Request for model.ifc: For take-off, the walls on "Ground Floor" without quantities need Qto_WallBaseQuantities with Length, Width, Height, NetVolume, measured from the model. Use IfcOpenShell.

First a look at what the model holds.

```python
import ifcopenshell
import ifcopenshell.util.element
import ifcopenshell.util.unit

model = ifcopenshell.open("model.ifc")
print(model.schema)
for unit_type in ("LENGTHUNIT", "AREAUNIT", "VOLUMEUNIT"):
    print(unit_type, ifcopenshell.util.unit.calculate_unit_scale(model, unit_type))
storey = next(s for s in model.by_type("IfcBuildingStorey") if s.Name == "Ground Floor")
walls = [e for e in ifcopenshell.util.element.get_decomposition(storey) if e.is_a("IfcWall")]
for e in sorted(walls, key=lambda e: e.id()):
    print(e.id(), e.is_a(), e.Name, list(ifcopenshell.util.element.get_psets(e, qtos_only=True)), sep=" | ")
```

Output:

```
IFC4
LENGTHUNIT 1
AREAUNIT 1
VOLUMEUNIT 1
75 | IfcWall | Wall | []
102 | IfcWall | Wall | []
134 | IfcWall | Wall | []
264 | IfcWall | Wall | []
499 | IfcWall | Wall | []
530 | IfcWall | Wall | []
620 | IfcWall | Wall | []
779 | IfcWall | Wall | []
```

```python
import ifcopenshell
import ifcopenshell.api.pset
import ifcopenshell.geom
import ifcopenshell.util.element
import ifcopenshell.util.shape
import ifcopenshell.util.unit

model = ifcopenshell.open("model.ifc")
unit_scale = ifcopenshell.util.unit.calculate_unit_scale(model)
volume_scale = ifcopenshell.util.unit.calculate_unit_scale(model, "VOLUMEUNIT")
settings = ifcopenshell.geom.settings()

storey = next(s for s in model.by_type("IfcBuildingStorey") if s.Name == "Ground Floor")
walls = [e for e in ifcopenshell.util.element.get_decomposition(storey) if e.is_a("IfcWall")]

for e in sorted(walls, key=lambda e: e.id()):
    if ifcopenshell.util.element.get_psets(e, qtos_only=True, should_inherit=False):
        continue
    # Geometry comes back in metres, in the element's own axes.
    shape = ifcopenshell.geom.create_shape(settings, e)
    values = {
        "Length": ifcopenshell.util.shape.get_x(shape.geometry) / unit_scale,
        "Width": ifcopenshell.util.shape.get_y(shape.geometry) / unit_scale,
        "Height": ifcopenshell.util.shape.get_z(shape.geometry) / unit_scale,
        "NetVolume": ifcopenshell.util.shape.get_volume(shape.geometry) / volume_scale,
    }
    qto = ifcopenshell.api.pset.add_qto(model, product=e, name="Qto_WallBaseQuantities")
    ifcopenshell.api.pset.edit_qto(model, qto=qto, properties=values)
    print(e.id(), {k: round(v, 3) for k, v in values.items()})

model.write("model_updated.ifc")
```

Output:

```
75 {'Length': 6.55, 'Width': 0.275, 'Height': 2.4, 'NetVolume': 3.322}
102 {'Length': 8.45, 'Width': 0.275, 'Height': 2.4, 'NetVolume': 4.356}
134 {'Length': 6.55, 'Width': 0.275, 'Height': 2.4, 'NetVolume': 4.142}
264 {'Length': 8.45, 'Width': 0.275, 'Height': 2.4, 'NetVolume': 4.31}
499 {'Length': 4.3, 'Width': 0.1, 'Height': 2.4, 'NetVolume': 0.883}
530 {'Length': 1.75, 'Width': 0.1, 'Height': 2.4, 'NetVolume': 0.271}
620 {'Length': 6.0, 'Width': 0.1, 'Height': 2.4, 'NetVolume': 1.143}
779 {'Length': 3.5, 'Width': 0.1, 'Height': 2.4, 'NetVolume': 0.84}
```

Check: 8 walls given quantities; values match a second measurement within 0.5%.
